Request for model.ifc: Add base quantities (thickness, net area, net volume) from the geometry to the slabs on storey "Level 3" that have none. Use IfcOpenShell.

First a look at what the model holds.

```python
import ifcopenshell
import ifcopenshell.util.element
import ifcopenshell.util.unit

model = ifcopenshell.open("model.ifc")
print(model.schema)
for unit_type in ("LENGTHUNIT", "AREAUNIT", "VOLUMEUNIT"):
    print(unit_type, ifcopenshell.util.unit.calculate_unit_scale(model, unit_type))
storey = next(s for s in model.by_type("IfcBuildingStorey") if s.Name == "Level 3")
slabs = [e for e in ifcopenshell.util.element.get_decomposition(storey) if e.is_a("IfcSlab")]
for e in sorted(slabs, key=lambda e: e.id()):
    print(e.id(), e.is_a(), e.Name, list(ifcopenshell.util.element.get_psets(e, qtos_only=True)), sep=" | ")
```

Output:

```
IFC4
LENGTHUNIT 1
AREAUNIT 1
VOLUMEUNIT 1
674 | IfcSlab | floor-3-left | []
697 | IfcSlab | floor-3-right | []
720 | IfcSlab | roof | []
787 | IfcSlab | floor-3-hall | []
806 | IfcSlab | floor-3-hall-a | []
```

```python
import ifcopenshell
import ifcopenshell.api.pset
import ifcopenshell.geom
import ifcopenshell.util.element
import ifcopenshell.util.shape
import ifcopenshell.util.unit

model = ifcopenshell.open("model.ifc")
unit_scale = ifcopenshell.util.unit.calculate_unit_scale(model)
area_scale = ifcopenshell.util.unit.calculate_unit_scale(model, "AREAUNIT")
volume_scale = ifcopenshell.util.unit.calculate_unit_scale(model, "VOLUMEUNIT")
settings = ifcopenshell.geom.settings()

storey = next(s for s in model.by_type("IfcBuildingStorey") if s.Name == "Level 3")
slabs = [e for e in ifcopenshell.util.element.get_decomposition(storey) if e.is_a("IfcSlab")]

for e in sorted(slabs, key=lambda e: e.id()):
    if ifcopenshell.util.element.get_psets(e, qtos_only=True, should_inherit=False):
        continue
    # Geometry comes back in metres, in the element's own axes.
    shape = ifcopenshell.geom.create_shape(settings, e)
    values = {
        "Width": ifcopenshell.util.shape.get_z(shape.geometry) / unit_scale,
        "NetArea": ifcopenshell.util.shape.get_footprint_area(shape.geometry) / area_scale,
        "NetVolume": ifcopenshell.util.shape.get_volume(shape.geometry) / volume_scale,
    }
    qto = ifcopenshell.api.pset.add_qto(model, product=e, name="Qto_SlabBaseQuantities")
    ifcopenshell.api.pset.edit_qto(model, qto=qto, properties=values)
    print(e.id(), {k: round(v, 3) for k, v in values.items()})

model.write("model_rev.ifc")
```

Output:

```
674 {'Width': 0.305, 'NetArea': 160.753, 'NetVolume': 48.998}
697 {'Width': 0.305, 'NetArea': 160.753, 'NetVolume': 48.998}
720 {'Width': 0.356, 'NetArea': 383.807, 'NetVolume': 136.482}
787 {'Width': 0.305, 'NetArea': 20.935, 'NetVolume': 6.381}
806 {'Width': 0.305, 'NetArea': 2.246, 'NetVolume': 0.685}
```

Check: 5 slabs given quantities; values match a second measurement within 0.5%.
